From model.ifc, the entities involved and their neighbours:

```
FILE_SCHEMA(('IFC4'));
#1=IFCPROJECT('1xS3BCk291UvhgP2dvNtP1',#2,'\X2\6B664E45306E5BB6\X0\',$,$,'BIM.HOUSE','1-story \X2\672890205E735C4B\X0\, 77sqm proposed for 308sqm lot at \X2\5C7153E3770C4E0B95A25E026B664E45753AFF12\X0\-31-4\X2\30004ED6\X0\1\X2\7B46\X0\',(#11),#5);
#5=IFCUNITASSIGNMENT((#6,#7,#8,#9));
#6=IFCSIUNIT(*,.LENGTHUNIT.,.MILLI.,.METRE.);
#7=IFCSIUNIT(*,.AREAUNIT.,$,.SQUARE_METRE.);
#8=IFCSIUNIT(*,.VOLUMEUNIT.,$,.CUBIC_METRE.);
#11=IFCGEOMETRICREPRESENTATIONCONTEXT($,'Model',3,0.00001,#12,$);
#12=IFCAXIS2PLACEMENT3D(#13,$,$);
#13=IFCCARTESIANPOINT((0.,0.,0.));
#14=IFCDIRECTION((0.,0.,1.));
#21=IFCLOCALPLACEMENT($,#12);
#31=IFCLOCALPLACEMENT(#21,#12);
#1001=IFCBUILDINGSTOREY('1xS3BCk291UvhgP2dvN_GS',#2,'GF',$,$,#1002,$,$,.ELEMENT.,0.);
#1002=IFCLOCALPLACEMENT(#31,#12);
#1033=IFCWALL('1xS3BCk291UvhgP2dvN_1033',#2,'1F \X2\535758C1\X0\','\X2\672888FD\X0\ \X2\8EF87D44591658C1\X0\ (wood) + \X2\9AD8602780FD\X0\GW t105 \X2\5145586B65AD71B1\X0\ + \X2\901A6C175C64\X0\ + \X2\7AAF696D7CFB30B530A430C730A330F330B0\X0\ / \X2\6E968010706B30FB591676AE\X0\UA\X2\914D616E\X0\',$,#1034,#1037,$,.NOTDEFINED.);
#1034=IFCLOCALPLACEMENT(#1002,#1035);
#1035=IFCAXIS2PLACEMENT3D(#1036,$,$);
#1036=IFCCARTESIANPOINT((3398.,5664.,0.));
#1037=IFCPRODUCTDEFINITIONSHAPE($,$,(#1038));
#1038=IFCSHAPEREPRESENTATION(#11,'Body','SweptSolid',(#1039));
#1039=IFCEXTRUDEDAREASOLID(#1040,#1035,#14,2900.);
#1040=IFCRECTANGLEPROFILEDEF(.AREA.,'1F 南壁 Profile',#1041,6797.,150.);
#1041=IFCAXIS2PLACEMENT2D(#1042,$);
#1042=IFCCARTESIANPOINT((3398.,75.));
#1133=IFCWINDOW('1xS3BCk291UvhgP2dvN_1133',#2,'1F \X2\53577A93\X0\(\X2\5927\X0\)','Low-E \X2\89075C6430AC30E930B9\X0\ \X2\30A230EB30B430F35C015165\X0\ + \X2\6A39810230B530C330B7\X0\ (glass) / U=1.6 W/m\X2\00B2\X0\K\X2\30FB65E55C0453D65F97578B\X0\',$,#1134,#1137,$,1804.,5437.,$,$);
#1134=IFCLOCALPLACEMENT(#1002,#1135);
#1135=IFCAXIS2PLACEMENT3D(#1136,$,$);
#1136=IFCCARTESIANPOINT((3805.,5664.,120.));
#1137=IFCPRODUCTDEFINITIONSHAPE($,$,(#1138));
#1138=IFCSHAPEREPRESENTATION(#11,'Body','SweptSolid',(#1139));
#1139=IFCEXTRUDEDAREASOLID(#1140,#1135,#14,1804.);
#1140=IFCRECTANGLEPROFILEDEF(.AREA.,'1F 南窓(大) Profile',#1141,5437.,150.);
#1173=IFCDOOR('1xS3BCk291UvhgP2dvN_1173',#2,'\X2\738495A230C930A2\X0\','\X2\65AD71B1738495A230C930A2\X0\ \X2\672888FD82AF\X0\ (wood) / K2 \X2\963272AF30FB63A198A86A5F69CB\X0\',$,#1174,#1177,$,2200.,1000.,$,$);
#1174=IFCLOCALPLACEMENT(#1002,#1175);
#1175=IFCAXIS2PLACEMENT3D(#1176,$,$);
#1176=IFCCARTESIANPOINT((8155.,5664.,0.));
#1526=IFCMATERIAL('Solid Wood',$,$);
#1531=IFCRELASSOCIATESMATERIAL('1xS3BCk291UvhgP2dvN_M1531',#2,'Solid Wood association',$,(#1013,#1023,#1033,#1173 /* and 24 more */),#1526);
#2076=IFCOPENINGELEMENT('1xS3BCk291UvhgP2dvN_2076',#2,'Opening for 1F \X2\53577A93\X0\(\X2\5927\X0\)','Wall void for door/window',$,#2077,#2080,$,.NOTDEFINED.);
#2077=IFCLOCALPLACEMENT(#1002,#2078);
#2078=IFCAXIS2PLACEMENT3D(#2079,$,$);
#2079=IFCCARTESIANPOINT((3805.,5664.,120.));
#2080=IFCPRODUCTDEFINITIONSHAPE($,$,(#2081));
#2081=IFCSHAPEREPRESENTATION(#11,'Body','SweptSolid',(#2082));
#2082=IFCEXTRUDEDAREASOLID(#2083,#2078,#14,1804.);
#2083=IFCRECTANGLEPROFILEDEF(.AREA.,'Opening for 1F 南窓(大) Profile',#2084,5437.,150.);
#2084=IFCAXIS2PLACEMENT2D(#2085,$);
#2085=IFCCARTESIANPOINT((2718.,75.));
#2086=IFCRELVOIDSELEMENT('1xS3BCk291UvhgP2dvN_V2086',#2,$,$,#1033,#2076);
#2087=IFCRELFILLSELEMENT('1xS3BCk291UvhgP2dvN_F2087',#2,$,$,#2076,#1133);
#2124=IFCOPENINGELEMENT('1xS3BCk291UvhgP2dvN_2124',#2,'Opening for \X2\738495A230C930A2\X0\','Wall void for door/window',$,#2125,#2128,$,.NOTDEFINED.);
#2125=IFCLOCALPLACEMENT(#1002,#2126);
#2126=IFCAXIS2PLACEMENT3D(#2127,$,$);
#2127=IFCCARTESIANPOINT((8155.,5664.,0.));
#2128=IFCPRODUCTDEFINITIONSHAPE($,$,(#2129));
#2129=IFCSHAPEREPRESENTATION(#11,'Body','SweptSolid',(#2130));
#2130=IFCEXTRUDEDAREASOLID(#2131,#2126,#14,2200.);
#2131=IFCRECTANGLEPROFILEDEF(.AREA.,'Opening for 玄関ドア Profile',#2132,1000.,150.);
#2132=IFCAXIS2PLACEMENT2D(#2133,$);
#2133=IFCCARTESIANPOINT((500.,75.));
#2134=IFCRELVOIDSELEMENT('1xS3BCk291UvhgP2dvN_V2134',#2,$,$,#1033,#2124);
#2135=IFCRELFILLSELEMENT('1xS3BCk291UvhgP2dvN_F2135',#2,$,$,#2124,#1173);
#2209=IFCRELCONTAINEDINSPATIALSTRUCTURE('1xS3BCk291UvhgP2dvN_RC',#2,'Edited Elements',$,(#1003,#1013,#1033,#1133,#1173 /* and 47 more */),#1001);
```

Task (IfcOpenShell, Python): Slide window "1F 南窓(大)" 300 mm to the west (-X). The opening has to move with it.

```python
import ifcopenshell
import ifcopenshell.api.geometry
import ifcopenshell.util.placement

model = ifcopenshell.open("model.ifc")

window = model.by_guid("1xS3BCk291UvhgP2dvN_1133")
opening = window.FillsVoids[0].RelatingOpeningElement
wall = opening.VoidsElements[0].RelatingBuildingElement

wall_matrix = ifcopenshell.util.placement.get_local_placement(wall.ObjectPlacement)
shift = wall_matrix[:3, 0] * -300.0
before = ifcopenshell.util.placement.get_local_placement(window.ObjectPlacement)[:3, 3].copy()

# The window is not placed relative to its opening, so move both.
for product in (opening, window):
    matrix = ifcopenshell.util.placement.get_local_placement(product.ObjectPlacement)
    matrix[:3, 3] += shift
    ifcopenshell.api.geometry.edit_object_placement(model, product=product, matrix=matrix, is_si=False)

after = ifcopenshell.util.placement.get_local_placement(window.ObjectPlacement)[:3, 3]
print("window moved by", (after - before).round(3) + 0.0)

model.write("model_updated.ifc")
```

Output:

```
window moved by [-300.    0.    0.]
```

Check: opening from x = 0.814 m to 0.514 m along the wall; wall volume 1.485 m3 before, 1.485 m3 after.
